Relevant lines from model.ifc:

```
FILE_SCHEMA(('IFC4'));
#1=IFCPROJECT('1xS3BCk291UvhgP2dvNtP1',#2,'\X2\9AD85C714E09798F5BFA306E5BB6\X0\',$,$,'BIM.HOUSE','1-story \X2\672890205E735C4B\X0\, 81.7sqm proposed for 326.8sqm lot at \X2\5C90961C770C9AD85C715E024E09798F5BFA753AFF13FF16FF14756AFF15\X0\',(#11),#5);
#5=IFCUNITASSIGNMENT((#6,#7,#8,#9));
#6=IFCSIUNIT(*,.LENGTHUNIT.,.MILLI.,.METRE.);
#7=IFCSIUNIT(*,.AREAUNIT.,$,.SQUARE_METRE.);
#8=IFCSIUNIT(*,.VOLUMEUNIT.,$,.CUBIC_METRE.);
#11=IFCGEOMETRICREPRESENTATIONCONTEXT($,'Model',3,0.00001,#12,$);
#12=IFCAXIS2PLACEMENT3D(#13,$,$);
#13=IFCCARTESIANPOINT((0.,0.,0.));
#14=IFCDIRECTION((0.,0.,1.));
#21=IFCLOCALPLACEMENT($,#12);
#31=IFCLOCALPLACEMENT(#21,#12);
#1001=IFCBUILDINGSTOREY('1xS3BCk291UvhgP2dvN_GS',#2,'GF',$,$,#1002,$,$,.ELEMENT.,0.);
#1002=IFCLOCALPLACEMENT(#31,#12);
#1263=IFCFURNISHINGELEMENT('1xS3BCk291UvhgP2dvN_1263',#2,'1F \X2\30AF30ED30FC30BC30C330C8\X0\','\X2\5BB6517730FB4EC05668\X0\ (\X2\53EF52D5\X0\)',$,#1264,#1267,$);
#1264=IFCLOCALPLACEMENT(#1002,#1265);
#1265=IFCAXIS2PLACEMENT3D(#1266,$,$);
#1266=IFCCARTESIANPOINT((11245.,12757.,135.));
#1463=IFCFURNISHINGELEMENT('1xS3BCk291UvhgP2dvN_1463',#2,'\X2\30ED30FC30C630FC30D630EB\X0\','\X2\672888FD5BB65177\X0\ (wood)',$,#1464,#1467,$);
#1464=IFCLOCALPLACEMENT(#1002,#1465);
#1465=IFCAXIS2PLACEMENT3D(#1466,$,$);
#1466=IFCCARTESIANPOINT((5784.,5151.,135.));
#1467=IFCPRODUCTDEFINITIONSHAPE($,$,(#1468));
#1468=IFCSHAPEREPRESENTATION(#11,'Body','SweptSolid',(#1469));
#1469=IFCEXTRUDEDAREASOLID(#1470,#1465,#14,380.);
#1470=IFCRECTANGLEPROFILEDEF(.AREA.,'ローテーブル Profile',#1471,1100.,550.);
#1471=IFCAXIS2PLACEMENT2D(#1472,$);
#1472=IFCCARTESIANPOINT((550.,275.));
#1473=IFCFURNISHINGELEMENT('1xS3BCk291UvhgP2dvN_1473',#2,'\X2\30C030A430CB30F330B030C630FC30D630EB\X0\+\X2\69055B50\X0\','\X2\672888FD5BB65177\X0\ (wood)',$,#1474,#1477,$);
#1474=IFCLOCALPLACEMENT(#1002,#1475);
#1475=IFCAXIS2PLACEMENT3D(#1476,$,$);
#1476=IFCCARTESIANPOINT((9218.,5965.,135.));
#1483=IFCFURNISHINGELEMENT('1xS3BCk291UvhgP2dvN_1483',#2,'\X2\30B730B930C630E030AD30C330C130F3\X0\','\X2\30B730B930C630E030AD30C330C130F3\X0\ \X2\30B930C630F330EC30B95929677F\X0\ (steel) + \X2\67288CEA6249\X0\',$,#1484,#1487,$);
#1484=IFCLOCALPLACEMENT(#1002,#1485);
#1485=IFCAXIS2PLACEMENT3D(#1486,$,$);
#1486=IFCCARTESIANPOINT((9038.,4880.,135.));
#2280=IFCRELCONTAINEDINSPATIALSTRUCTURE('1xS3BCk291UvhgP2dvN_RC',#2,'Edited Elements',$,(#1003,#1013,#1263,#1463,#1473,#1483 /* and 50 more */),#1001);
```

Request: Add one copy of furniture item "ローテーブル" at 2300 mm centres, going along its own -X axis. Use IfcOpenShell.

```python
import ifcopenshell
import ifcopenshell.api.geometry
import ifcopenshell.api.root
import ifcopenshell.util.element
import ifcopenshell.util.placement

model = ifcopenshell.open("model.ifc")


def reuse_history(source, copy):
    """copy_class also copies each property set's owner history, people and application; keep the originals."""
    for rel in copy.IsDefinedBy:
        if rel.is_a("IfcRelDefinesByProperties") and (history := rel.RelatingPropertyDefinition.OwnerHistory):
            rel.RelatingPropertyDefinition.OwnerHistory = source.OwnerHistory
            ifcopenshell.util.element.remove_deep2(model, history)


source = model.by_guid("1xS3BCk291UvhgP2dvN_1463")
base = ifcopenshell.util.placement.get_local_placement(source.ObjectPlacement)
step = -base[:3, 0] * 2300.0

for i in range(1, 2):
    copy = ifcopenshell.api.root.copy_class(model, product=source)
    copy.Representation = ifcopenshell.util.element.copy_deep(
        model, source.Representation, exclude=["IfcGeometricRepresentationContext", "IfcRepresentationMap"]
    )
    reuse_history(source, copy)
    matrix = base.copy()
    matrix[:3, 3] += i * step
    print("added at", matrix[:3, 3].round(3) + 0.0)
    ifcopenshell.api.geometry.edit_object_placement(model, product=copy, matrix=matrix, is_si=False)

model.write("model_v2.ifc")
```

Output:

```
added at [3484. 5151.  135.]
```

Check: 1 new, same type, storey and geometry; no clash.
